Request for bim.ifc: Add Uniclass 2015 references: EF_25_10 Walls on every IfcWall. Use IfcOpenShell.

First a look at what the model holds.

```python
import ifcopenshell

model = ifcopenshell.open("bim.ifc")
print(model.schema)
print("classifications:", [c.Name for c in model.by_type("IfcClassification")])
for ifc_class in ("IfcDoor", "IfcRoof", "IfcStair", "IfcWall", "IfcWindow"):
    print(ifc_class, len(model.by_type(ifc_class)))
```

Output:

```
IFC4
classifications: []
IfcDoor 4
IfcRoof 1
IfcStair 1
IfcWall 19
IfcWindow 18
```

```python
import ifcopenshell
import ifcopenshell.api.classification

model = ifcopenshell.open("bim.ifc")

system = ifcopenshell.api.classification.add_classification(model, classification="Uniclass 2015")

codes = {
    "IfcWall": ("EF_25_10", "Walls"),
}
for ifc_class, (code, name) in codes.items():
    products = model.by_type(ifc_class)
    ifcopenshell.api.classification.add_reference(
        model, products=products, classification=system, identification=code, name=name
    )
    print(code, len(products))

model.write("bim_updated.ifc")
```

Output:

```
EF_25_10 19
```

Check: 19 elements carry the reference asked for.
